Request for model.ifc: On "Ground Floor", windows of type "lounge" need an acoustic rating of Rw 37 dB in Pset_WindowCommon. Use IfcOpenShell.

First a look at what the model holds.

```python
import ifcopenshell
import ifcopenshell.util.element

model = ifcopenshell.open("model.ifc")
print(model.schema)
storey = next(s for s in model.by_type("IfcBuildingStorey") if s.Name == "Ground Floor")
windows = [e for e in ifcopenshell.util.element.get_decomposition(storey) if e.is_a("IfcWindow")]
seen = {}
for e in windows:
    element_type = ifcopenshell.util.element.get_type(e)
    key = (element_type.Name if element_type != e and element_type else None, ifcopenshell.util.element.get_pset(e, "Pset_WindowCommon", "AcousticRating"))
    seen[key] = seen.get(key, 0) + 1
for (name, value), count in sorted(seen.items(), key=str):
    print(count, "x", name, "|", value)
```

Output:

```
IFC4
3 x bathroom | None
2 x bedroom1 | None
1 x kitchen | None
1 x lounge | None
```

```python
import ifcopenshell
import ifcopenshell.api.pset
import ifcopenshell.util.element

model = ifcopenshell.open("model.ifc")

storey = next(s for s in model.by_type("IfcBuildingStorey") if s.Name == "Ground Floor")
windows = [e for e in ifcopenshell.util.element.get_decomposition(storey) if e.is_a("IfcWindow")]

count = 0
for e in windows:
    element_type = ifcopenshell.util.element.get_type(e)
    if element_type in (None, e) or element_type.Name != "lounge":
        continue
    # add_pset returns the element's existing set when there is one.
    pset = ifcopenshell.api.pset.add_pset(model, product=e, name="Pset_WindowCommon")
    ifcopenshell.api.pset.edit_pset(model, pset=pset, properties={"AcousticRating": "Rw 37 dB"})
    count += 1

print(count, "windows updated")

model.write("model_v2.ifc")
```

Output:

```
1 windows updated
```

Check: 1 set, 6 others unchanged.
